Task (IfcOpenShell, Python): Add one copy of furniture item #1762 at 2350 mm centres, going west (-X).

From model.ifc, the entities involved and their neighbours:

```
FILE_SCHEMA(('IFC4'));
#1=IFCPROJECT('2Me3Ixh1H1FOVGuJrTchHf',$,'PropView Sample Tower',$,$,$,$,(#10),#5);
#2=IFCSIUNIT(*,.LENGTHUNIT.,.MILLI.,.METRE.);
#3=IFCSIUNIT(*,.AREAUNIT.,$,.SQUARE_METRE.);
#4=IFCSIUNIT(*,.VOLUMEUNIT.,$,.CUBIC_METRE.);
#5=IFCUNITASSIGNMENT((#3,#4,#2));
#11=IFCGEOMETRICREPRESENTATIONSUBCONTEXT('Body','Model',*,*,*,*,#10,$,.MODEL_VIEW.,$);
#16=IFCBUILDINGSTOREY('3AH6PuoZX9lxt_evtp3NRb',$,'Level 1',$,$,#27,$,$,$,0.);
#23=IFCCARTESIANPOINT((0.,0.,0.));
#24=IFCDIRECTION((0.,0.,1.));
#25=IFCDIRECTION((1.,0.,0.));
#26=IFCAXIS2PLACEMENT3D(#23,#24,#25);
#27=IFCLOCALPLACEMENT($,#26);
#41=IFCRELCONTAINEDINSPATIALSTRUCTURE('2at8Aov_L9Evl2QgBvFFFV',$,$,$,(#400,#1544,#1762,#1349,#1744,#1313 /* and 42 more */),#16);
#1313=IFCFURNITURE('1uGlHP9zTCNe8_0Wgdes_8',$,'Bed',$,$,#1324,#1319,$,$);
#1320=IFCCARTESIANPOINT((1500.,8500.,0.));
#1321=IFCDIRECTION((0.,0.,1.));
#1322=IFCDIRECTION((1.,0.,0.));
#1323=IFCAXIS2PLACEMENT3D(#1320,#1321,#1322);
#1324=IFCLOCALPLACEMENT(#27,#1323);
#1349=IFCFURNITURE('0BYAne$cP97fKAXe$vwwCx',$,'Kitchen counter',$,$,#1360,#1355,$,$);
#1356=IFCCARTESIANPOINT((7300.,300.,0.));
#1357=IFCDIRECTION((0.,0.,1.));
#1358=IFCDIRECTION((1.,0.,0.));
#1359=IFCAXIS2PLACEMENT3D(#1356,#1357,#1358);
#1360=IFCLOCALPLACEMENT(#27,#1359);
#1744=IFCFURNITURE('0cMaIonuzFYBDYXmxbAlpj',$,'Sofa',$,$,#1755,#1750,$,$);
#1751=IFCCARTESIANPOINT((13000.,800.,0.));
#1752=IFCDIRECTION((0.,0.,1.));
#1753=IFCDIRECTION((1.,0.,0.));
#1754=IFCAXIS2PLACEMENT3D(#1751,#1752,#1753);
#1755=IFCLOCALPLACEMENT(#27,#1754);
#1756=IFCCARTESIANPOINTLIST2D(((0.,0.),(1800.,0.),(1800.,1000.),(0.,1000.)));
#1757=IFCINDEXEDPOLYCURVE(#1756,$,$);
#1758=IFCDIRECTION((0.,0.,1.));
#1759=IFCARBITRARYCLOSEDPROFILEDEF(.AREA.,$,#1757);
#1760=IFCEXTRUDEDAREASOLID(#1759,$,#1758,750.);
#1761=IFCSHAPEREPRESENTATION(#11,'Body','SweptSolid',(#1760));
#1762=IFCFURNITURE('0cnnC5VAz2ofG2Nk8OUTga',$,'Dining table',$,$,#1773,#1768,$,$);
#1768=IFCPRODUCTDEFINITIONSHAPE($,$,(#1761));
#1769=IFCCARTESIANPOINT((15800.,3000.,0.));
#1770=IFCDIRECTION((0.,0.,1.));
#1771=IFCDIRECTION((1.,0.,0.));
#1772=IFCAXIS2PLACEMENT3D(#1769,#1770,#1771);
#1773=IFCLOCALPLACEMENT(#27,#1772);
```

```python
import numpy as np
import ifcopenshell
import ifcopenshell.api.geometry
import ifcopenshell.api.root
import ifcopenshell.util.element
import ifcopenshell.util.placement
import ifcopenshell.util.unit

model = ifcopenshell.open("model.ifc")
unit_scale = ifcopenshell.util.unit.calculate_unit_scale(model)

source = model.by_id(1762)
base = ifcopenshell.util.placement.get_local_placement(source.ObjectPlacement)
step = np.array([-1.0, 0.0, 0.0]) * 2.35 / unit_scale

for i in range(1, 2):
    copy = ifcopenshell.api.root.copy_class(model, product=source)
    copy.Representation = ifcopenshell.util.element.copy_deep(
        model, source.Representation, exclude=["IfcGeometricRepresentationContext", "IfcRepresentationMap"]
    )
    matrix = base.copy()
    matrix[:3, 3] += i * step
    print("added at", matrix[:3, 3].round(3) + 0.0)
    ifcopenshell.api.geometry.edit_object_placement(model, product=copy, matrix=matrix, is_si=False)

model.write("model_updated.ifc")
```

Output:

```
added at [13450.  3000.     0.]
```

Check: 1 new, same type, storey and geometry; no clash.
